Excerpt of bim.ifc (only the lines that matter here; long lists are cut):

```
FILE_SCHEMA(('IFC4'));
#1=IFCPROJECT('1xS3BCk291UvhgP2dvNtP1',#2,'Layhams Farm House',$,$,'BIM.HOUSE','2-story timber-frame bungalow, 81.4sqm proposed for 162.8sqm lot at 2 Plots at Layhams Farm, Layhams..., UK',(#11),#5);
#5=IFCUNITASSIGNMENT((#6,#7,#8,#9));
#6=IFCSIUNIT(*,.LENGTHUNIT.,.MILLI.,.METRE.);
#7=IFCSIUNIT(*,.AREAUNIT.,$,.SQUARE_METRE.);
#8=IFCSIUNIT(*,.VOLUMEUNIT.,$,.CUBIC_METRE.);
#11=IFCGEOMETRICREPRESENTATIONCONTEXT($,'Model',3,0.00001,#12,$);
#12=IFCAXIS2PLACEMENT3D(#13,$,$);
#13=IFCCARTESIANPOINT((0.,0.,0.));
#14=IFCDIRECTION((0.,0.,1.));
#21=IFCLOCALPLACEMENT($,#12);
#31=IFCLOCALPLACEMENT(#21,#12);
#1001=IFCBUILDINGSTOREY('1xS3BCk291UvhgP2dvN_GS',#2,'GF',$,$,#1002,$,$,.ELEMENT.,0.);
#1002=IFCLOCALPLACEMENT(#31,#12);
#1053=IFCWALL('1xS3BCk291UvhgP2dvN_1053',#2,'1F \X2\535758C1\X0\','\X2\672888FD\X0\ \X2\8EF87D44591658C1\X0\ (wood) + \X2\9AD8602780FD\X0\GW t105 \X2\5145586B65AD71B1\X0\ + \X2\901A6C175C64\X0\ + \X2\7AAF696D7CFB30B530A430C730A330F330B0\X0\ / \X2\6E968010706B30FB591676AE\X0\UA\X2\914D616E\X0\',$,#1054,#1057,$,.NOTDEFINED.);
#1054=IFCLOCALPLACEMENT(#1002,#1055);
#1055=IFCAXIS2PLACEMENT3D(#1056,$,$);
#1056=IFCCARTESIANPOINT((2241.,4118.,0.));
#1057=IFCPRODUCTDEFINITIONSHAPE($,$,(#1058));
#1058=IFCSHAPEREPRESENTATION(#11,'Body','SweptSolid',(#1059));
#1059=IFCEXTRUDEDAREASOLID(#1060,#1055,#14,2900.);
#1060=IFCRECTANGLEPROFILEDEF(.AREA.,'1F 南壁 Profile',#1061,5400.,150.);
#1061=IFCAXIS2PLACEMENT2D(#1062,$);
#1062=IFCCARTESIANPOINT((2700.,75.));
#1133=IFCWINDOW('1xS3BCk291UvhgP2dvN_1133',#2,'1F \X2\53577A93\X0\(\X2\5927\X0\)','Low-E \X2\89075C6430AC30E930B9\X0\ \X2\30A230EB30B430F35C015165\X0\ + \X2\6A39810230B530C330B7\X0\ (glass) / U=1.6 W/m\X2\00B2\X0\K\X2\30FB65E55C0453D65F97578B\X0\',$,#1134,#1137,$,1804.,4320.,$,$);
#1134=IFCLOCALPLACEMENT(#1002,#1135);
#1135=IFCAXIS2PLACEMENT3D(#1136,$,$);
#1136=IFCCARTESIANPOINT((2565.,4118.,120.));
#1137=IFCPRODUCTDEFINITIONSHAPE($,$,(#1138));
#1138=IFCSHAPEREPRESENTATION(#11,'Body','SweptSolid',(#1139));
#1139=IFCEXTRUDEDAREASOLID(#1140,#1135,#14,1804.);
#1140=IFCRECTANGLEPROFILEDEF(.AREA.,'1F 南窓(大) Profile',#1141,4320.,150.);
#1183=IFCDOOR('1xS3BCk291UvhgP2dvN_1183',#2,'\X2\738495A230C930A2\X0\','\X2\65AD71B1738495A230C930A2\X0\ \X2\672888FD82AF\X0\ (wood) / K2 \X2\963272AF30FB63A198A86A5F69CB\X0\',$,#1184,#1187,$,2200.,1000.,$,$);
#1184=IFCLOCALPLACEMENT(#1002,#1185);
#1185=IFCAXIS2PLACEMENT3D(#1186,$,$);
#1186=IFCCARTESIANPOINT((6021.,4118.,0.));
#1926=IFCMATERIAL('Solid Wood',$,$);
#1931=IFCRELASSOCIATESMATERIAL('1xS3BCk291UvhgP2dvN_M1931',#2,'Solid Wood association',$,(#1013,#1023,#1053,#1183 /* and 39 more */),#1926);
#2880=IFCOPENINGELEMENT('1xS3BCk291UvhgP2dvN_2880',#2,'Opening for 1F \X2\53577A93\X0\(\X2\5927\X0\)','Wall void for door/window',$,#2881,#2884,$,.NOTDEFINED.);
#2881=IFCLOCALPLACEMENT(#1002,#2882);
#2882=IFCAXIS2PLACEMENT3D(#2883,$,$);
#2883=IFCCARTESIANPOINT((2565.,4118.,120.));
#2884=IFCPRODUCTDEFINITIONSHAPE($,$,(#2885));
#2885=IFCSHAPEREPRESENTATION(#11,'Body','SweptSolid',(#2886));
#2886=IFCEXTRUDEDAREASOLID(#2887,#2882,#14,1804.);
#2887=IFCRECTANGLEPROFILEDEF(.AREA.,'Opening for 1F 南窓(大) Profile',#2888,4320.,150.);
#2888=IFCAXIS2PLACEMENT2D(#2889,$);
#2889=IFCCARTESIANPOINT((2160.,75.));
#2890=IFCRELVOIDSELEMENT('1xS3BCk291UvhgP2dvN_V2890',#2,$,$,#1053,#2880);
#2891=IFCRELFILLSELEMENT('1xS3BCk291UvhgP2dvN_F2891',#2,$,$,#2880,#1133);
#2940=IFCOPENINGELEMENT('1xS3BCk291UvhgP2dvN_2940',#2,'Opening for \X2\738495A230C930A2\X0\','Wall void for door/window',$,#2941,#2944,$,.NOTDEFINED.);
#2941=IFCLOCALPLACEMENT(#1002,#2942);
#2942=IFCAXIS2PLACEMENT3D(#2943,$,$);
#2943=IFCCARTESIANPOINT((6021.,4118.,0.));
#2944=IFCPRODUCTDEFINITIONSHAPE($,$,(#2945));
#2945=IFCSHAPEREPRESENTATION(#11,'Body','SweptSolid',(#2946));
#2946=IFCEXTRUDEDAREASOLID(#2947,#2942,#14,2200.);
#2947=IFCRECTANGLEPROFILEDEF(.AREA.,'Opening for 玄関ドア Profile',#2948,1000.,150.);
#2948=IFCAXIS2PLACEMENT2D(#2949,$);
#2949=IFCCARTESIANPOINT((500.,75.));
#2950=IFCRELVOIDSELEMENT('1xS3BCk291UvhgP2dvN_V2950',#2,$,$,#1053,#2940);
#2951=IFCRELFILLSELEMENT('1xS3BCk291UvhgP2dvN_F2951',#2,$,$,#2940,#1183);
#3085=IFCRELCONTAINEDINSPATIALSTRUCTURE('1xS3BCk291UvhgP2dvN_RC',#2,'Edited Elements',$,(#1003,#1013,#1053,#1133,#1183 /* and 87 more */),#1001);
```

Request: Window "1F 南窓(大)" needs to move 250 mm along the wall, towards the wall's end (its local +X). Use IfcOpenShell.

```python
import ifcopenshell
import ifcopenshell.api.geometry
import ifcopenshell.util.placement

model = ifcopenshell.open("bim.ifc")

window = model.by_id(1133)
opening = window.FillsVoids[0].RelatingOpeningElement
wall = opening.VoidsElements[0].RelatingBuildingElement

wall_matrix = ifcopenshell.util.placement.get_local_placement(wall.ObjectPlacement)
shift = wall_matrix[:3, 0] * 250.0
before = ifcopenshell.util.placement.get_local_placement(window.ObjectPlacement)[:3, 3].copy()

# The window is not placed relative to its opening, so move both.
for product in (opening, window):
    matrix = ifcopenshell.util.placement.get_local_placement(product.ObjectPlacement)
    matrix[:3, 3] += shift
    ifcopenshell.api.geometry.edit_object_placement(model, product=product, matrix=matrix, is_si=False)

after = ifcopenshell.util.placement.get_local_placement(window.ObjectPlacement)[:3, 3]
print("window moved by", (after - before).round(3) + 0.0)

model.write("bim-out.ifc")
```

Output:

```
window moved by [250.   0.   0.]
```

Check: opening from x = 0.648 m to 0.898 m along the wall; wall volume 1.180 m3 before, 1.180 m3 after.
